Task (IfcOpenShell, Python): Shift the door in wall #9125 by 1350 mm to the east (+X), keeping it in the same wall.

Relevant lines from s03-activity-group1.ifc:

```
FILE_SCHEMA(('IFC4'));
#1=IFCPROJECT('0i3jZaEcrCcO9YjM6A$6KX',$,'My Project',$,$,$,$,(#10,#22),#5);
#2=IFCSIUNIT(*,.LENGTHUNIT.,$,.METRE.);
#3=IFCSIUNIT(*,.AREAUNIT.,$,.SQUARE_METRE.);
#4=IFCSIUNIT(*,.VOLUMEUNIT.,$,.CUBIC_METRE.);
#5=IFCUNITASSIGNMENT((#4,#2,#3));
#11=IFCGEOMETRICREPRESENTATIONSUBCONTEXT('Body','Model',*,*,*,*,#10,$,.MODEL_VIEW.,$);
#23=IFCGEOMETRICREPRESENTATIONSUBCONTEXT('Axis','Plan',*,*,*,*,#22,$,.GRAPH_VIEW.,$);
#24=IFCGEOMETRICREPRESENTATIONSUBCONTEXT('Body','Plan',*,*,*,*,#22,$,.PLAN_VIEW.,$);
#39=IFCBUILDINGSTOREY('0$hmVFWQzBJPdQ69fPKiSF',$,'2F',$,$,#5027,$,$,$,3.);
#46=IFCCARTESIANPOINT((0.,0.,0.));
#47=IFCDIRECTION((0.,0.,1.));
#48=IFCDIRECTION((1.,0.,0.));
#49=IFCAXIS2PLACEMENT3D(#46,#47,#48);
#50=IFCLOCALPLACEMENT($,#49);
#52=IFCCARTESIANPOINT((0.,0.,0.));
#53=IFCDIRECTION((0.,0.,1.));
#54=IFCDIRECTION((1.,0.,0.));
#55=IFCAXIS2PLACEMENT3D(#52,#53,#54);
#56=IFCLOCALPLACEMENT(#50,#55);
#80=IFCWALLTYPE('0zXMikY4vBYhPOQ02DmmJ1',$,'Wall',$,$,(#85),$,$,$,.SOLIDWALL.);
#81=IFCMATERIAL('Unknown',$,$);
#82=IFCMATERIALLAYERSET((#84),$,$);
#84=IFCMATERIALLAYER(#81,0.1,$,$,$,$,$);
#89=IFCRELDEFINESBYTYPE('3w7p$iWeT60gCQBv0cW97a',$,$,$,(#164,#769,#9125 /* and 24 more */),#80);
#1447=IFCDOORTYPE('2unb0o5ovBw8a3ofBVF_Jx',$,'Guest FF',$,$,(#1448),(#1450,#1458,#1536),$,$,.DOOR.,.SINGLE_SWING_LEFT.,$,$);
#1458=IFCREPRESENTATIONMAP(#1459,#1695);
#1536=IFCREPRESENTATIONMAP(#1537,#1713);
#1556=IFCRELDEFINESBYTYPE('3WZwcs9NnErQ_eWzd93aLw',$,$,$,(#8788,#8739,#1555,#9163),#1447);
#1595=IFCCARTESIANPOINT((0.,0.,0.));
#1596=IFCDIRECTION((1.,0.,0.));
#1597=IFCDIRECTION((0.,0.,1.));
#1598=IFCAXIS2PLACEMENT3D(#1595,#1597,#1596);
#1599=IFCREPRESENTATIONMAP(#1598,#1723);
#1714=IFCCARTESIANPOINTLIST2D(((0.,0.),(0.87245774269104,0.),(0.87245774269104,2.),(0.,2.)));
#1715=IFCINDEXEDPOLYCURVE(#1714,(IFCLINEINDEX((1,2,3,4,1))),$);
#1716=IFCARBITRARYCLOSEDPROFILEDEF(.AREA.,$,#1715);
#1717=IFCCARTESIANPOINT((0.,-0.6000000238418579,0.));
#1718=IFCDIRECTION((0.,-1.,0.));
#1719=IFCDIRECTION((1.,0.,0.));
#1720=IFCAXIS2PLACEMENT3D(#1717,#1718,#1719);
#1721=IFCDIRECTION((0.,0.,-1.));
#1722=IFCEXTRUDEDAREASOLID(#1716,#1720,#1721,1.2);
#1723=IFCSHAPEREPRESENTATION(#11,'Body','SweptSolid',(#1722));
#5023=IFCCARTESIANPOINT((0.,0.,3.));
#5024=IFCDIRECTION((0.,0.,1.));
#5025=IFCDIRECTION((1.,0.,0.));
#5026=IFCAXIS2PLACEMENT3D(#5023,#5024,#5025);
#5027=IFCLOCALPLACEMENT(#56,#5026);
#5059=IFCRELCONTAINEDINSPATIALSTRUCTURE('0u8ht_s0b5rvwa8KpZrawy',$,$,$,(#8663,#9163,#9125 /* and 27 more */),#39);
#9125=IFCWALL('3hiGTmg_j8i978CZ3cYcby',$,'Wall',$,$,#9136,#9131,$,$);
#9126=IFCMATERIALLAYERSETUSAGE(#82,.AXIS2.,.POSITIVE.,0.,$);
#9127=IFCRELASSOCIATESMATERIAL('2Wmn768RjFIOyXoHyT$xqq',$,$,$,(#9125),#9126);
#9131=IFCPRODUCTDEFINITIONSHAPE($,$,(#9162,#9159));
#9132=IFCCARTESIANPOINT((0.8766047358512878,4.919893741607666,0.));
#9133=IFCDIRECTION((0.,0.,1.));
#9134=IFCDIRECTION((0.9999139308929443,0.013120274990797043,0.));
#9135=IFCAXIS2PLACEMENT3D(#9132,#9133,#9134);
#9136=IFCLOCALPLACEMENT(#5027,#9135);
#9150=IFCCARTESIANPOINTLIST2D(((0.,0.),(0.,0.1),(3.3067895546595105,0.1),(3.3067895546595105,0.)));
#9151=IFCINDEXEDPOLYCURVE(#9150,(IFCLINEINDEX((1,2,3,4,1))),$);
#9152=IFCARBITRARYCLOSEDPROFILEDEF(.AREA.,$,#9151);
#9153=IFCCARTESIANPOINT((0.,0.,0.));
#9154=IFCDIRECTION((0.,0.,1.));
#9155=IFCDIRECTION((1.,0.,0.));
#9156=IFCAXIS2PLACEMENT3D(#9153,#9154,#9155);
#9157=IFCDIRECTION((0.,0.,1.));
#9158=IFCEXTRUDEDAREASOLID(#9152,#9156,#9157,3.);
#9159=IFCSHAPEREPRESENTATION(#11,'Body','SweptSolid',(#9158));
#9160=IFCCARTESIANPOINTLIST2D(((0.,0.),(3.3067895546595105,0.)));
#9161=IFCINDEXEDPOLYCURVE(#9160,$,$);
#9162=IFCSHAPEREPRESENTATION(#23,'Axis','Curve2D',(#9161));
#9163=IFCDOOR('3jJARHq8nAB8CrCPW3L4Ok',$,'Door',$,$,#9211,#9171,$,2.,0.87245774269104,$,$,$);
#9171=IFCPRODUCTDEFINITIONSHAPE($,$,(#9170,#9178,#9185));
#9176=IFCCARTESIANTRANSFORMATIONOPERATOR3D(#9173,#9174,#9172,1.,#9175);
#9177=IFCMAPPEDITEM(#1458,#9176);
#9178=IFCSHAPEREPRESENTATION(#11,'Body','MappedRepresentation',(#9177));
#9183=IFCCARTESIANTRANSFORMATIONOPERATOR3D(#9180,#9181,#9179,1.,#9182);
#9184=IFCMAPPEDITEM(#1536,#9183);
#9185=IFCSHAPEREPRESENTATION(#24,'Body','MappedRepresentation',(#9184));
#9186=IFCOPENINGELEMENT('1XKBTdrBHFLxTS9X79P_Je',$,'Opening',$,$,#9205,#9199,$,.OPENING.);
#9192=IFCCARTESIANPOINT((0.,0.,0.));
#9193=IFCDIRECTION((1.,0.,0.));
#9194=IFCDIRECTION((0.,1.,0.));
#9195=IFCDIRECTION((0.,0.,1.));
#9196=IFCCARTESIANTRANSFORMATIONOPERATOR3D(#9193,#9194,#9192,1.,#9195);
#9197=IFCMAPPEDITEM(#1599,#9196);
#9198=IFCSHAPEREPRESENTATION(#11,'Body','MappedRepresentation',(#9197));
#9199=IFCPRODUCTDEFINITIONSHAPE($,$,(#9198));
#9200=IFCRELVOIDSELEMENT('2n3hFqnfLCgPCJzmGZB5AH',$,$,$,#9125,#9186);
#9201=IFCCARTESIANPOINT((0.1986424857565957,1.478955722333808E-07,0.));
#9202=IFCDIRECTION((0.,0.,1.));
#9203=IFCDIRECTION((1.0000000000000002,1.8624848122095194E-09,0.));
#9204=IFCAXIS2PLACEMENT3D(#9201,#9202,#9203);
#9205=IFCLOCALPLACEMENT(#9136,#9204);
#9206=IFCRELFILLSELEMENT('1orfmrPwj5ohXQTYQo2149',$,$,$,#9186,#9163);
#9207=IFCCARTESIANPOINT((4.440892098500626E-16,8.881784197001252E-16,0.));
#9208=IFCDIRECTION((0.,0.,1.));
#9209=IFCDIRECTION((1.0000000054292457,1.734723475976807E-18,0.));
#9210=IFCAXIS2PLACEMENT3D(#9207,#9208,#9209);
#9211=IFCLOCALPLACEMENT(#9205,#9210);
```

```python
import ifcopenshell
import ifcopenshell.api.geometry
import ifcopenshell.util.placement
import ifcopenshell.util.unit

model = ifcopenshell.open("s03-activity-group1.ifc")
unit_scale = ifcopenshell.util.unit.calculate_unit_scale(model)

door = model.by_id(9163)
opening = door.FillsVoids[0].RelatingOpeningElement
wall = opening.VoidsElements[0].RelatingBuildingElement

wall_matrix = ifcopenshell.util.placement.get_local_placement(wall.ObjectPlacement)
shift = wall_matrix[:3, 0] * 1.35 / unit_scale
before = ifcopenshell.util.placement.get_local_placement(door.ObjectPlacement)[:3, 3].copy()

# The door is placed relative to its opening, so it follows when the opening moves.
matrix = ifcopenshell.util.placement.get_local_placement(opening.ObjectPlacement)
matrix[:3, 3] += shift
ifcopenshell.api.geometry.edit_object_placement(
    model, product=opening, matrix=matrix, is_si=False, should_transform_children=True
)

after = ifcopenshell.util.placement.get_local_placement(door.ObjectPlacement)[:3, 3]
print("door moved by", (after - before).round(3) + 0.0)

model.write("s03-activity-group1_rev.ifc")
```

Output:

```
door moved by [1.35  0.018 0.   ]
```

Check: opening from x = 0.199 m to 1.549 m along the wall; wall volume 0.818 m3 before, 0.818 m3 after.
